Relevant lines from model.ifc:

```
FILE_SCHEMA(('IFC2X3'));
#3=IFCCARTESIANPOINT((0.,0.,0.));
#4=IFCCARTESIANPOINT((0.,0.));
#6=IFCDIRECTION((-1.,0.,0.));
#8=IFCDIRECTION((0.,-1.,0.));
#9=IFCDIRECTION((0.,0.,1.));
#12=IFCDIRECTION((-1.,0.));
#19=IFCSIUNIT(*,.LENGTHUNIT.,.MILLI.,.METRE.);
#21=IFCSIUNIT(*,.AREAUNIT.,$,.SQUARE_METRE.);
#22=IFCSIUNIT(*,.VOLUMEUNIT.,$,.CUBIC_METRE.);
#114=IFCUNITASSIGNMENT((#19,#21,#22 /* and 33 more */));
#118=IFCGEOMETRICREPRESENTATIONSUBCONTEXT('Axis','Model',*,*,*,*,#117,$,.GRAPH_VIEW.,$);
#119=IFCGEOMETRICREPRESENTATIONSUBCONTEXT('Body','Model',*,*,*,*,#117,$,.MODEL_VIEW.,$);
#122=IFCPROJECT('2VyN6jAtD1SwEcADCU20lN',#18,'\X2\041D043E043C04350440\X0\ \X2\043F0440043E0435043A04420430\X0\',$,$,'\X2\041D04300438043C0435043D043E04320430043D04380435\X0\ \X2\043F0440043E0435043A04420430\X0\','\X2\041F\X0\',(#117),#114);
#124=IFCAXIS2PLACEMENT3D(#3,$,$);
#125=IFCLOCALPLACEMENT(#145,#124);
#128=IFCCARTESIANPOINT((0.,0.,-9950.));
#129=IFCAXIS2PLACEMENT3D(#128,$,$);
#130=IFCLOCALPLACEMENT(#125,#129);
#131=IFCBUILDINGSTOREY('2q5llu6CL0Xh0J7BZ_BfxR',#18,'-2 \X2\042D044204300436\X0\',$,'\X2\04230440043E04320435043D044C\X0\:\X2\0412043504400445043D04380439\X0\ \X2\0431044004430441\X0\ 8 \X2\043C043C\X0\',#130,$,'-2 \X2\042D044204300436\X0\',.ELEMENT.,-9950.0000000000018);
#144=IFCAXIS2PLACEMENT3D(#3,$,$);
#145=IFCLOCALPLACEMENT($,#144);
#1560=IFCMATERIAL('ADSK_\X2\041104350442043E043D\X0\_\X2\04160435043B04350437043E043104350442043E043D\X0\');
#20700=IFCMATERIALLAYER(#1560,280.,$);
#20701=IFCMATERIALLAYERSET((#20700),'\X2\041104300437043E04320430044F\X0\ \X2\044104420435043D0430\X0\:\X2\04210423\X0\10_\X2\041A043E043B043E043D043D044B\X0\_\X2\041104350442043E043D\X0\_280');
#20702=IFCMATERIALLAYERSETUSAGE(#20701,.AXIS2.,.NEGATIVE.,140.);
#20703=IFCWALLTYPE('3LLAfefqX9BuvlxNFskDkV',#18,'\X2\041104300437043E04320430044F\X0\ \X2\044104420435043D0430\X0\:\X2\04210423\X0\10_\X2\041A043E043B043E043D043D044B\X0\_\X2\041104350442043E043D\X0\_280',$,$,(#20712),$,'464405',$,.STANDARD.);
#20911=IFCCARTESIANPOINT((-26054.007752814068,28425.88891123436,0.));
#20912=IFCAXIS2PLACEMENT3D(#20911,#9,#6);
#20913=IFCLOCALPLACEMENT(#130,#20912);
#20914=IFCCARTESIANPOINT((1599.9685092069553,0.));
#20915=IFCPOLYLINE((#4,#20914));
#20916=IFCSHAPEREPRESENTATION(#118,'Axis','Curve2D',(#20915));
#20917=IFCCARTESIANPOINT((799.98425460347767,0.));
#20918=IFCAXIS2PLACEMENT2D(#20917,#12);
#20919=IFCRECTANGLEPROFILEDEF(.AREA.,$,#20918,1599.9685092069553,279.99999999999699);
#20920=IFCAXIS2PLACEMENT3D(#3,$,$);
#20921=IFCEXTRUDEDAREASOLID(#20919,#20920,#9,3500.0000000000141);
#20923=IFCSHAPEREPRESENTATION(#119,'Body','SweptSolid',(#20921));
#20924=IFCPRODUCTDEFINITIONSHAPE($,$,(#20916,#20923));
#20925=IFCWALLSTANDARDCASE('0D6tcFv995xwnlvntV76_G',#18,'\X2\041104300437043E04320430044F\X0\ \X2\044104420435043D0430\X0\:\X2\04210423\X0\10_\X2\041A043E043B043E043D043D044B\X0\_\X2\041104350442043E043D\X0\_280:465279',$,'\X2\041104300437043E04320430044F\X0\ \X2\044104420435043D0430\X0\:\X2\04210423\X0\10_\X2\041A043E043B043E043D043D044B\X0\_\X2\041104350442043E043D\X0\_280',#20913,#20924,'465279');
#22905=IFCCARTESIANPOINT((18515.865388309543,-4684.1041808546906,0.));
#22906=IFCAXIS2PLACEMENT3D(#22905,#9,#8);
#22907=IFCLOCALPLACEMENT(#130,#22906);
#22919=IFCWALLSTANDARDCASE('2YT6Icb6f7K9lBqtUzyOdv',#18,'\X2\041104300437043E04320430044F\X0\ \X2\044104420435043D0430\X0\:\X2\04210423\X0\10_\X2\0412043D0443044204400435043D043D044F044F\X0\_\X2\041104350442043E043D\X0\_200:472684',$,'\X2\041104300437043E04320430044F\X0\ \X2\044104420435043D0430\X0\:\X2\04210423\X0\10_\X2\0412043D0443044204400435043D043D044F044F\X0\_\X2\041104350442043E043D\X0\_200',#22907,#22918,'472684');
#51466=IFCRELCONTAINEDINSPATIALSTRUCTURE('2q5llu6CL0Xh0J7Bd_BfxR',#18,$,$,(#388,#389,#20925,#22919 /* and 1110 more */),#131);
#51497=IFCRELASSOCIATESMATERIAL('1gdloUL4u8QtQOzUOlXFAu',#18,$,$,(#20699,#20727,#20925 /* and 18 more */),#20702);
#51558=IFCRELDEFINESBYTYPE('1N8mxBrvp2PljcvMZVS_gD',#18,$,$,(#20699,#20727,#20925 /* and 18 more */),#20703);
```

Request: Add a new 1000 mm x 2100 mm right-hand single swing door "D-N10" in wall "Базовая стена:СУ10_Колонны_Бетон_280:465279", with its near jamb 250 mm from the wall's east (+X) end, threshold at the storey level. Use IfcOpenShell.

```python
import numpy as np
import ifcopenshell
import ifcopenshell.api.feature
import ifcopenshell.api.geometry
import ifcopenshell.api.root
import ifcopenshell.api.spatial
import ifcopenshell.api.type
import ifcopenshell.geom
import ifcopenshell.util.element
import ifcopenshell.util.placement
import ifcopenshell.util.representation
import ifcopenshell.util.shape
import ifcopenshell.util.unit

model = ifcopenshell.open("model.ifc")
unit_scale = ifcopenshell.util.unit.calculate_unit_scale(model)
settings = ifcopenshell.geom.settings()


def volume(element):
    """Net volume in cubic metres, openings subtracted."""
    shape = ifcopenshell.geom.create_shape(settings, element)
    return ifcopenshell.util.shape.get_volume(shape.geometry)


wall = model.by_guid("0D6tcFv995xwnlvntV76_G")
storey = ifcopenshell.util.element.get_container(wall, ifc_class="IfcBuildingStorey")
context = ifcopenshell.util.representation.get_context(model, "Model", "Body", "MODEL_VIEW")
before = volume(wall)

width, height, from_end, sill = 1, 2.1, 0.25, 0.0  # metres

# The wall runs along its own X axis, and the end named is its -X end.
wall_shape = ifcopenshell.geom.create_shape(settings, wall)
x, y, z = ifcopenshell.util.shape.get_vertices(wall_shape.geometry).T
start = x.min() + from_end
face, thickness = float(y.min()), float(y.max() - y.min())
wall_matrix = ifcopenshell.util.placement.get_local_placement(wall.ObjectPlacement)
level = ifcopenshell.util.placement.get_local_placement(storey.ObjectPlacement)[2, 3]


def in_wall(x, y):
    """Placement at x, y metres in the wall's axes, at sill height."""
    matrix = wall_matrix.copy()
    matrix[:, 3] = wall_matrix @ np.array([x / unit_scale, y / unit_scale, 0.0, 1.0])
    matrix[2, 3] = level + sill / unit_scale
    return matrix


# Opening: a box that overshoots both wall faces by 50 mm.
opening = ifcopenshell.api.root.create_entity(model, ifc_class="IfcOpeningElement")
box = ifcopenshell.api.geometry.add_wall_representation(
    model, context=context, length=width, height=height, thickness=thickness + 0.1
)
ifcopenshell.api.geometry.assign_representation(model, product=opening, representation=box)
ifcopenshell.api.geometry.edit_object_placement(model, product=opening, matrix=in_wall(start, face - 0.05), is_si=False)
ifcopenshell.api.feature.add_feature(model, feature=opening, element=wall)

door = ifcopenshell.api.root.create_entity(model, ifc_class="IfcDoor", name="D-N10")
door.OverallWidth, door.OverallHeight = width / unit_scale, height / unit_scale
body = ifcopenshell.api.geometry.add_door_representation(
    model,
    context=context,
    overall_width=door.OverallWidth,
    overall_height=door.OverallHeight,
    operation_type="SINGLE_SWING_RIGHT",
    lining_properties={"LiningDepth": thickness / unit_scale, "ThresholdDepth": thickness / unit_scale},
)
ifcopenshell.api.geometry.assign_representation(model, product=door, representation=body)
ifcopenshell.api.spatial.assign_container(model, products=[door], relating_structure=storey)
fills = ifcopenshell.api.feature.add_filling(model, opening=opening, element=door)
fills.OwnerHistory = door.OwnerHistory  # required in IFC2X3

# IFC2X3 keeps the operation on the door style.
style = ifcopenshell.api.root.create_entity(model, ifc_class="IfcDoorStyle", name="D-N10")
style.OperationType, style.ConstructionType = "SINGLE_SWING_RIGHT", "NOTDEFINED"
style.ParameterTakesPrecedence = style.Sizeable = False
ifcopenshell.api.type.assign_type(model, related_objects=[door], relating_type=style)

# The lining spans the wall, so the door starts at the wall face.
ifcopenshell.api.geometry.edit_object_placement(model, product=door, matrix=in_wall(start, face), is_si=False)

after = volume(wall)

print(f"wall volume {before:.3f} -> {after:.3f} m3")

model.write("model_edited.ifc")
```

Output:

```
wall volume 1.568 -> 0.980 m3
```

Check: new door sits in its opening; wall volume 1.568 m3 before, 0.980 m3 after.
